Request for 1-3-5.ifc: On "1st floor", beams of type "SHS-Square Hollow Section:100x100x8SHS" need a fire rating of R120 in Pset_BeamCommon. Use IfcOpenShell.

First a look at what the model holds.

```python
import ifcopenshell
import ifcopenshell.util.element

model = ifcopenshell.open("1-3-5.ifc")
print(model.schema)
storey = next(s for s in model.by_type("IfcBuildingStorey") if s.Name == "1st floor")
beams = [e for e in ifcopenshell.util.element.get_decomposition(storey) if e.is_a("IfcBeam")]
seen = {}
for e in beams:
    element_type = ifcopenshell.util.element.get_type(e)
    key = (element_type.Name if element_type != e and element_type else None, ifcopenshell.util.element.get_pset(e, "Pset_BeamCommon", "FireRating"))
    seen[key] = seen.get(key, 0) + 1
for (name, value), count in sorted(seen.items(), key=str):
    print(count, "x", name, "|", value)
```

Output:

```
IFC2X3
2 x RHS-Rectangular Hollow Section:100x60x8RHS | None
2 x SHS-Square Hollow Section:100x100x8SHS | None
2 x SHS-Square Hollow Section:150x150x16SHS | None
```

```python
import ifcopenshell
import ifcopenshell.api.pset
import ifcopenshell.util.element

model = ifcopenshell.open("1-3-5.ifc")

storey = next(s for s in model.by_type("IfcBuildingStorey") if s.Name == "1st floor")
beams = [e for e in ifcopenshell.util.element.get_decomposition(storey) if e.is_a("IfcBeam")]

count = 0
for e in beams:
    element_type = ifcopenshell.util.element.get_type(e)
    if element_type in (None, e) or element_type.Name != "SHS-Square Hollow Section:100x100x8SHS":
        continue
    # add_pset returns the element's existing set when there is one.
    pset = ifcopenshell.api.pset.add_pset(model, product=e, name="Pset_BeamCommon")
    ifcopenshell.api.pset.edit_pset(model, pset=pset, properties={"FireRating": "R120"})
    count += 1

print(count, "beams updated")

model.write("1-3-5-out.ifc")
```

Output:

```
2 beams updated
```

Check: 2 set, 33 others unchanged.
